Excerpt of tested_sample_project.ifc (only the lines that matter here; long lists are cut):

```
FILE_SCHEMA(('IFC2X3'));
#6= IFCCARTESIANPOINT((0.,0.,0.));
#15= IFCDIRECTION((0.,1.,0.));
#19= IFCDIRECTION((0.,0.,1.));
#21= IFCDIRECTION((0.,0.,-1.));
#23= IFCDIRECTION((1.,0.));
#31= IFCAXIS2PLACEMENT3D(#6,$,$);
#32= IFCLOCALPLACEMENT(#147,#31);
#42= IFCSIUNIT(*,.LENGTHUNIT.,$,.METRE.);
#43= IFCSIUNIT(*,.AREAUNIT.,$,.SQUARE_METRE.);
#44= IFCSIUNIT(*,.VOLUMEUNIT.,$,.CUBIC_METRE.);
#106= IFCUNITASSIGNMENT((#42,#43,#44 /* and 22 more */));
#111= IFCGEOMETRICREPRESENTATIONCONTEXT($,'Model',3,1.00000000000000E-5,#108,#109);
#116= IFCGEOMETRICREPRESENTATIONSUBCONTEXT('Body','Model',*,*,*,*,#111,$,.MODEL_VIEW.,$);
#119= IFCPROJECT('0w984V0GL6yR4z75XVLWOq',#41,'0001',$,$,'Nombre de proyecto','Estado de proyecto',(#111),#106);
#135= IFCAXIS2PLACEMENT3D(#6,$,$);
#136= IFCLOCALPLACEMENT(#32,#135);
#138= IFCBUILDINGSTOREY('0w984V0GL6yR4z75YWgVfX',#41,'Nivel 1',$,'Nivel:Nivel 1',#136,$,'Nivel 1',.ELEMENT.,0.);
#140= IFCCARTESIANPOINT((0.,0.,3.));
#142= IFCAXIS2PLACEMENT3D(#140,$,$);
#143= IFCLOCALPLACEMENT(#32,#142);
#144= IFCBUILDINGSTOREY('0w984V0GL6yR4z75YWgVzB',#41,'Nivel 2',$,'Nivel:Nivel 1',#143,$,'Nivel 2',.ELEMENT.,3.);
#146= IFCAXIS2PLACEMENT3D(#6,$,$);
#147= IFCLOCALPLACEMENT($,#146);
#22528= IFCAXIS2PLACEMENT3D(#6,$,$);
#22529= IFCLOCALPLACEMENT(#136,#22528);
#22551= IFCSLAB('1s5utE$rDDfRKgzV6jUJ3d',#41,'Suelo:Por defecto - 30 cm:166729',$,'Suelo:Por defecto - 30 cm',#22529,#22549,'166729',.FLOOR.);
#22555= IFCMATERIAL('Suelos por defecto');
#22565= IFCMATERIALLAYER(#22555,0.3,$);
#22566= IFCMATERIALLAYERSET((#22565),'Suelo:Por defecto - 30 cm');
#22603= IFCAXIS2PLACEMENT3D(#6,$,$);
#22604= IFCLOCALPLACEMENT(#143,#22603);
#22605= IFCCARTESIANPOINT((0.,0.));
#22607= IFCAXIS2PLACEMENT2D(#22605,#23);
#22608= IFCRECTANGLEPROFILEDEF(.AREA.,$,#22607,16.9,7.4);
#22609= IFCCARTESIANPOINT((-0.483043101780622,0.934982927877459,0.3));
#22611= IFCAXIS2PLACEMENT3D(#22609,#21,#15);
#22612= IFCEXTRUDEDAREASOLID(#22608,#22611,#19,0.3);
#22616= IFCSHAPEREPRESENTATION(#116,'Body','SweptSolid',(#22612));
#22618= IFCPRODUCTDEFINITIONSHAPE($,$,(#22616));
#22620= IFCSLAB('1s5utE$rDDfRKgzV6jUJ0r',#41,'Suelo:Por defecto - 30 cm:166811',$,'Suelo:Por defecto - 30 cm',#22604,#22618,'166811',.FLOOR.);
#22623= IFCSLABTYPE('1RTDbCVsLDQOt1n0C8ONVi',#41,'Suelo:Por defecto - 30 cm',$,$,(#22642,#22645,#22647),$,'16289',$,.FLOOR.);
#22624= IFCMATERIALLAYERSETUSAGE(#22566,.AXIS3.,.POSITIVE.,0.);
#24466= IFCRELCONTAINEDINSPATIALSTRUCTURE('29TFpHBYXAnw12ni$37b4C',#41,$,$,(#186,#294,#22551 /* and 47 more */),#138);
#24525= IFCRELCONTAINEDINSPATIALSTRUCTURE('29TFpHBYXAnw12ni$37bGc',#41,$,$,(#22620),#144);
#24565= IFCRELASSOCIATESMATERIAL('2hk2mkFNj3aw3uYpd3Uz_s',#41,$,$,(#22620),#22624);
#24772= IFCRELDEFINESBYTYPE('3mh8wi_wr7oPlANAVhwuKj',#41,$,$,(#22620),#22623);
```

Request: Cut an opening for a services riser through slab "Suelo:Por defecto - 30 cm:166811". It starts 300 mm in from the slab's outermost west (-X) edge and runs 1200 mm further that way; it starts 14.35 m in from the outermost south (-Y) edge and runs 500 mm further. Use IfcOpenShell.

```python
import numpy as np
import ifcopenshell
import ifcopenshell.api.feature
import ifcopenshell.api.geometry
import ifcopenshell.api.root
import ifcopenshell.geom
import ifcopenshell.util.placement
import ifcopenshell.util.representation
import ifcopenshell.util.shape
import ifcopenshell.util.unit

model = ifcopenshell.open("tested_sample_project.ifc")
unit_scale = ifcopenshell.util.unit.calculate_unit_scale(model)
settings = ifcopenshell.geom.settings()


def volume(element):
    """Net volume in cubic metres, openings subtracted."""
    shape = ifcopenshell.geom.create_shape(settings, element)
    return ifcopenshell.util.shape.get_volume(shape.geometry)


slab = model.by_guid("1s5utE$rDDfRKgzV6jUJ0r")
before = volume(slab)

# Extent in the slab's own axes, in metres. The edges named are its -X and -Y sides.
slab_shape = ifcopenshell.geom.create_shape(settings, slab)
vertices = ifcopenshell.util.shape.get_vertices(slab_shape.geometry)
x_min, y_min, bottom = vertices.min(axis=0)
top = vertices[:, 2].max()

opening = ifcopenshell.api.root.create_entity(model, ifc_class="IfcOpeningElement", name="Services riser opening")
context = ifcopenshell.util.representation.get_context(model, "Model", "Body", "MODEL_VIEW")
width, depth = 1.2, 0.5
outline = [(0.0, 0.0), (width, 0.0), (width, depth), (0.0, depth), (0.0, 0.0)]
# Overshoot both faces by 50 mm so the cut is clean.
shape = ifcopenshell.api.geometry.add_slab_representation(
    model, context=context, depth=top - bottom + 0.1, polyline=outline
)
ifcopenshell.api.geometry.assign_representation(model, product=opening, representation=shape)

matrix = ifcopenshell.util.placement.get_local_placement(slab.ObjectPlacement)
matrix[:, 3] = matrix @ np.append(np.array([x_min + 0.3, y_min + 14.35, bottom - 0.05]) / unit_scale, 1.0)
ifcopenshell.api.geometry.edit_object_placement(model, product=opening, matrix=matrix, is_si=False)
ifcopenshell.api.feature.add_feature(model, feature=opening, element=slab)

after = volume(slab)

print(f"slab volume {before:.3f} -> {after:.3f} m3")

model.write("tested_sample_project-out.ifc")
```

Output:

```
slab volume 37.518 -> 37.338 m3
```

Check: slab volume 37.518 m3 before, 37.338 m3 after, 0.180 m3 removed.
